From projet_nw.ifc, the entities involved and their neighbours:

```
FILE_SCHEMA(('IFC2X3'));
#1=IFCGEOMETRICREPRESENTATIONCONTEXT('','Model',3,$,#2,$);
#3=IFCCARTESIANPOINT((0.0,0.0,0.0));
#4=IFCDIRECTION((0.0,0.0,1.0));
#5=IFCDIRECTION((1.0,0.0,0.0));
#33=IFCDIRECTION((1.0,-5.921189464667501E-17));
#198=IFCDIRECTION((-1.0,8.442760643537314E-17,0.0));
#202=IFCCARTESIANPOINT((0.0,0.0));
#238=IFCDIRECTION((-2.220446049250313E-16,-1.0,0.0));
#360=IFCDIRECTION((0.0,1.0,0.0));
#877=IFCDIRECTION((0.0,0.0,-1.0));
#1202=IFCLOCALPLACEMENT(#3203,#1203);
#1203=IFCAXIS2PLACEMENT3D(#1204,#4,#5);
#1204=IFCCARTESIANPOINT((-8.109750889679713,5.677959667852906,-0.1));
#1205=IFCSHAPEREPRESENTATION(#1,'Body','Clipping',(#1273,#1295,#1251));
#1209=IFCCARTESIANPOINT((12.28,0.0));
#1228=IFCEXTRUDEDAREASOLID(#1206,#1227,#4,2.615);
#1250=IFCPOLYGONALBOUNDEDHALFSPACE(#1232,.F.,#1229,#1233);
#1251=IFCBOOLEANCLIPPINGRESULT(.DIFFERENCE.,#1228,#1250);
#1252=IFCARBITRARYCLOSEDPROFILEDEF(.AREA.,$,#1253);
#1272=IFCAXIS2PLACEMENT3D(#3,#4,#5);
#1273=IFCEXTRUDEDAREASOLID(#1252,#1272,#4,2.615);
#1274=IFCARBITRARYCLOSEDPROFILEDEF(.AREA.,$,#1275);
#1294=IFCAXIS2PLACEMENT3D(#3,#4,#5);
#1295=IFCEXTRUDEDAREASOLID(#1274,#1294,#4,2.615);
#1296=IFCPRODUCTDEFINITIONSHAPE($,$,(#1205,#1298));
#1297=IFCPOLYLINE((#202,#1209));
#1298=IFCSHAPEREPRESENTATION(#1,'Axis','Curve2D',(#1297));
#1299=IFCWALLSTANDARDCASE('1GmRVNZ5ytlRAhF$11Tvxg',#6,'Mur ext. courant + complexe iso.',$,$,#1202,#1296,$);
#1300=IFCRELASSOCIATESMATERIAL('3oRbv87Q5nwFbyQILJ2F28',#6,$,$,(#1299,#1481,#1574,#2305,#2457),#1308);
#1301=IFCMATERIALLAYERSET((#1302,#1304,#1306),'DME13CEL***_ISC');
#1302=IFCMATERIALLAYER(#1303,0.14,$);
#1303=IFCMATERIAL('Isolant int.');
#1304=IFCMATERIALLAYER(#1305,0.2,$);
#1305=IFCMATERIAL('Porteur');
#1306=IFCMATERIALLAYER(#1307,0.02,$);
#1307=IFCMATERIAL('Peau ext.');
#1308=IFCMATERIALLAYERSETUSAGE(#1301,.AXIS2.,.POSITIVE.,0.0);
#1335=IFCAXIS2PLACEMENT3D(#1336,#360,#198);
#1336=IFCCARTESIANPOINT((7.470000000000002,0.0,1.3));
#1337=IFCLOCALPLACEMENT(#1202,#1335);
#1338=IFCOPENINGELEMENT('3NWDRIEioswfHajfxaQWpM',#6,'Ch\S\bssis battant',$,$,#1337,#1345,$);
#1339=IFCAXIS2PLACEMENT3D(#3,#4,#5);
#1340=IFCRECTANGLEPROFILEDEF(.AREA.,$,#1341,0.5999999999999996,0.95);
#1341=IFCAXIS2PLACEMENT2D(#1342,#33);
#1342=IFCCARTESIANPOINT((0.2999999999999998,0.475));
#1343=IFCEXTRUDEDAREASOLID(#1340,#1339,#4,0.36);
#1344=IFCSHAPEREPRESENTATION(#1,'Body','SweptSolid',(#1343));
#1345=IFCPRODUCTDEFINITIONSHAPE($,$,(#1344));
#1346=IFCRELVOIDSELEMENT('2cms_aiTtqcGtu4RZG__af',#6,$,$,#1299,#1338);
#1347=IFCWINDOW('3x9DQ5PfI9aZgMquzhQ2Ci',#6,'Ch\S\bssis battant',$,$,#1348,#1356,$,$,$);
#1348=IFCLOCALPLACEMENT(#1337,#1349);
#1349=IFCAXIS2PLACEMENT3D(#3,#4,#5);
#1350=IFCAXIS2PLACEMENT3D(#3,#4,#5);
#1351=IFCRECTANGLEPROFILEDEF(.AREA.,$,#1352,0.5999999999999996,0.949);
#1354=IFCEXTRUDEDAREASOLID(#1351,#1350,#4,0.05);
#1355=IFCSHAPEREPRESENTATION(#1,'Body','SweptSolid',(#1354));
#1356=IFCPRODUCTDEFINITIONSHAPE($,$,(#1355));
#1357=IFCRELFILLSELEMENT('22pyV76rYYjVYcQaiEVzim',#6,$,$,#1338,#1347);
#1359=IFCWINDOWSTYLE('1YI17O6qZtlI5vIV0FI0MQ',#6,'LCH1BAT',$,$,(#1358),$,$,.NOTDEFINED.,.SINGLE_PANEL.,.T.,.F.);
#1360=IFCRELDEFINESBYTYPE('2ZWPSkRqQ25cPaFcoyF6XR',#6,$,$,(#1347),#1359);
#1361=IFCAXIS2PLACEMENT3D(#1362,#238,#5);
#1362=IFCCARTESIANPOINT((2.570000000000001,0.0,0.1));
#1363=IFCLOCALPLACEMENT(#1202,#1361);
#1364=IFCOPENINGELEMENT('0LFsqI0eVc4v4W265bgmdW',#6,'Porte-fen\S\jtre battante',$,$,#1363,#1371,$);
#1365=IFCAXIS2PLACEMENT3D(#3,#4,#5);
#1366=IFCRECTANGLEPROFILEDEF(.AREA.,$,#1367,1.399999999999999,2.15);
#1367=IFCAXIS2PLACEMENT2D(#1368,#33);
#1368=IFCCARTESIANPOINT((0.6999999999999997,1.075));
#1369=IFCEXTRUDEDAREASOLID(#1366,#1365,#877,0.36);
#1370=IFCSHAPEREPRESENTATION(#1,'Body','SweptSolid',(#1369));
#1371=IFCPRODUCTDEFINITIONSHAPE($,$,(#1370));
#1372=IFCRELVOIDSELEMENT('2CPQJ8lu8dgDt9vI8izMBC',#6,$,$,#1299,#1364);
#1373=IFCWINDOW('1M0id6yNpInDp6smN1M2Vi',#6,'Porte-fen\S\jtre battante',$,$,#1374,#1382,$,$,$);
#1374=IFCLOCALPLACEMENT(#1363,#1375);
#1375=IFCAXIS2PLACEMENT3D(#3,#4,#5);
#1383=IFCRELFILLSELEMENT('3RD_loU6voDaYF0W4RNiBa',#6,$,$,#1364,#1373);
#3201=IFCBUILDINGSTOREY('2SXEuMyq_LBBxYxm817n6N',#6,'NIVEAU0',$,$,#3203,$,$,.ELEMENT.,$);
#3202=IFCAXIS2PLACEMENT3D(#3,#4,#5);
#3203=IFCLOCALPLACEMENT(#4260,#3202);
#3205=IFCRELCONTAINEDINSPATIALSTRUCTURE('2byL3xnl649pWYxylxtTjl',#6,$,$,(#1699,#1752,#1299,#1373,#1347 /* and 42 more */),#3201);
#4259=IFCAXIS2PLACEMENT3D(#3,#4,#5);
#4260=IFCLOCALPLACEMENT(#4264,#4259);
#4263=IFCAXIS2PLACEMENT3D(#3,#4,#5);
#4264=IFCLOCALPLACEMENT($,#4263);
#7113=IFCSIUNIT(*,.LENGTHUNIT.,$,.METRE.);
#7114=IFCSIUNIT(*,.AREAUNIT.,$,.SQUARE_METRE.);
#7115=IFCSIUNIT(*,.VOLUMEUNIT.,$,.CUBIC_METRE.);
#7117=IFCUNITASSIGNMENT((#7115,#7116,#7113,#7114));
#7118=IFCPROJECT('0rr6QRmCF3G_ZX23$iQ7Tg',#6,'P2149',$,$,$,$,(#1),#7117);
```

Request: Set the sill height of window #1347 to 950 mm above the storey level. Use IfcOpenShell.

```python
import numpy as np
import ifcopenshell
import ifcopenshell.api.geometry
import ifcopenshell.geom
import ifcopenshell.util.element
import ifcopenshell.util.placement
import ifcopenshell.util.shape
import ifcopenshell.util.unit

model = ifcopenshell.open("projet_nw.ifc")
unit_scale = ifcopenshell.util.unit.calculate_unit_scale(model)

window = model.by_guid("3x9DQ5PfI9aZgMquzhQ2Ci")
opening = window.FillsVoids[0].RelatingOpeningElement
storey = ifcopenshell.util.element.get_container(window, ifc_class="IfcBuildingStorey")
level = ifcopenshell.util.placement.get_local_placement(storey.ObjectPlacement)[2, 3]

# The opening's origin need not be at the sill, so measure its lowest point.
shape = ifcopenshell.geom.create_shape(ifcopenshell.geom.settings(), opening)
bottom = ifcopenshell.util.shape.get_shape_bottom_elevation(shape, shape.geometry) / unit_scale
dz = level + 0.95 / unit_scale - bottom

shift = np.array([0.0, 0.0, dz])
# The window is placed relative to its opening, so it follows when the opening moves.
matrix = ifcopenshell.util.placement.get_local_placement(opening.ObjectPlacement)
matrix[:3, 3] += shift
ifcopenshell.api.geometry.edit_object_placement(
    model, product=opening, matrix=matrix, is_si=False, should_transform_children=True
)

print(f"moved by {dz * unit_scale:+.3f} m")

model.write("projet_nw_v2.ifc")
```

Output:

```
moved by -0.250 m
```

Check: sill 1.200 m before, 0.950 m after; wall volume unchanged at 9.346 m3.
